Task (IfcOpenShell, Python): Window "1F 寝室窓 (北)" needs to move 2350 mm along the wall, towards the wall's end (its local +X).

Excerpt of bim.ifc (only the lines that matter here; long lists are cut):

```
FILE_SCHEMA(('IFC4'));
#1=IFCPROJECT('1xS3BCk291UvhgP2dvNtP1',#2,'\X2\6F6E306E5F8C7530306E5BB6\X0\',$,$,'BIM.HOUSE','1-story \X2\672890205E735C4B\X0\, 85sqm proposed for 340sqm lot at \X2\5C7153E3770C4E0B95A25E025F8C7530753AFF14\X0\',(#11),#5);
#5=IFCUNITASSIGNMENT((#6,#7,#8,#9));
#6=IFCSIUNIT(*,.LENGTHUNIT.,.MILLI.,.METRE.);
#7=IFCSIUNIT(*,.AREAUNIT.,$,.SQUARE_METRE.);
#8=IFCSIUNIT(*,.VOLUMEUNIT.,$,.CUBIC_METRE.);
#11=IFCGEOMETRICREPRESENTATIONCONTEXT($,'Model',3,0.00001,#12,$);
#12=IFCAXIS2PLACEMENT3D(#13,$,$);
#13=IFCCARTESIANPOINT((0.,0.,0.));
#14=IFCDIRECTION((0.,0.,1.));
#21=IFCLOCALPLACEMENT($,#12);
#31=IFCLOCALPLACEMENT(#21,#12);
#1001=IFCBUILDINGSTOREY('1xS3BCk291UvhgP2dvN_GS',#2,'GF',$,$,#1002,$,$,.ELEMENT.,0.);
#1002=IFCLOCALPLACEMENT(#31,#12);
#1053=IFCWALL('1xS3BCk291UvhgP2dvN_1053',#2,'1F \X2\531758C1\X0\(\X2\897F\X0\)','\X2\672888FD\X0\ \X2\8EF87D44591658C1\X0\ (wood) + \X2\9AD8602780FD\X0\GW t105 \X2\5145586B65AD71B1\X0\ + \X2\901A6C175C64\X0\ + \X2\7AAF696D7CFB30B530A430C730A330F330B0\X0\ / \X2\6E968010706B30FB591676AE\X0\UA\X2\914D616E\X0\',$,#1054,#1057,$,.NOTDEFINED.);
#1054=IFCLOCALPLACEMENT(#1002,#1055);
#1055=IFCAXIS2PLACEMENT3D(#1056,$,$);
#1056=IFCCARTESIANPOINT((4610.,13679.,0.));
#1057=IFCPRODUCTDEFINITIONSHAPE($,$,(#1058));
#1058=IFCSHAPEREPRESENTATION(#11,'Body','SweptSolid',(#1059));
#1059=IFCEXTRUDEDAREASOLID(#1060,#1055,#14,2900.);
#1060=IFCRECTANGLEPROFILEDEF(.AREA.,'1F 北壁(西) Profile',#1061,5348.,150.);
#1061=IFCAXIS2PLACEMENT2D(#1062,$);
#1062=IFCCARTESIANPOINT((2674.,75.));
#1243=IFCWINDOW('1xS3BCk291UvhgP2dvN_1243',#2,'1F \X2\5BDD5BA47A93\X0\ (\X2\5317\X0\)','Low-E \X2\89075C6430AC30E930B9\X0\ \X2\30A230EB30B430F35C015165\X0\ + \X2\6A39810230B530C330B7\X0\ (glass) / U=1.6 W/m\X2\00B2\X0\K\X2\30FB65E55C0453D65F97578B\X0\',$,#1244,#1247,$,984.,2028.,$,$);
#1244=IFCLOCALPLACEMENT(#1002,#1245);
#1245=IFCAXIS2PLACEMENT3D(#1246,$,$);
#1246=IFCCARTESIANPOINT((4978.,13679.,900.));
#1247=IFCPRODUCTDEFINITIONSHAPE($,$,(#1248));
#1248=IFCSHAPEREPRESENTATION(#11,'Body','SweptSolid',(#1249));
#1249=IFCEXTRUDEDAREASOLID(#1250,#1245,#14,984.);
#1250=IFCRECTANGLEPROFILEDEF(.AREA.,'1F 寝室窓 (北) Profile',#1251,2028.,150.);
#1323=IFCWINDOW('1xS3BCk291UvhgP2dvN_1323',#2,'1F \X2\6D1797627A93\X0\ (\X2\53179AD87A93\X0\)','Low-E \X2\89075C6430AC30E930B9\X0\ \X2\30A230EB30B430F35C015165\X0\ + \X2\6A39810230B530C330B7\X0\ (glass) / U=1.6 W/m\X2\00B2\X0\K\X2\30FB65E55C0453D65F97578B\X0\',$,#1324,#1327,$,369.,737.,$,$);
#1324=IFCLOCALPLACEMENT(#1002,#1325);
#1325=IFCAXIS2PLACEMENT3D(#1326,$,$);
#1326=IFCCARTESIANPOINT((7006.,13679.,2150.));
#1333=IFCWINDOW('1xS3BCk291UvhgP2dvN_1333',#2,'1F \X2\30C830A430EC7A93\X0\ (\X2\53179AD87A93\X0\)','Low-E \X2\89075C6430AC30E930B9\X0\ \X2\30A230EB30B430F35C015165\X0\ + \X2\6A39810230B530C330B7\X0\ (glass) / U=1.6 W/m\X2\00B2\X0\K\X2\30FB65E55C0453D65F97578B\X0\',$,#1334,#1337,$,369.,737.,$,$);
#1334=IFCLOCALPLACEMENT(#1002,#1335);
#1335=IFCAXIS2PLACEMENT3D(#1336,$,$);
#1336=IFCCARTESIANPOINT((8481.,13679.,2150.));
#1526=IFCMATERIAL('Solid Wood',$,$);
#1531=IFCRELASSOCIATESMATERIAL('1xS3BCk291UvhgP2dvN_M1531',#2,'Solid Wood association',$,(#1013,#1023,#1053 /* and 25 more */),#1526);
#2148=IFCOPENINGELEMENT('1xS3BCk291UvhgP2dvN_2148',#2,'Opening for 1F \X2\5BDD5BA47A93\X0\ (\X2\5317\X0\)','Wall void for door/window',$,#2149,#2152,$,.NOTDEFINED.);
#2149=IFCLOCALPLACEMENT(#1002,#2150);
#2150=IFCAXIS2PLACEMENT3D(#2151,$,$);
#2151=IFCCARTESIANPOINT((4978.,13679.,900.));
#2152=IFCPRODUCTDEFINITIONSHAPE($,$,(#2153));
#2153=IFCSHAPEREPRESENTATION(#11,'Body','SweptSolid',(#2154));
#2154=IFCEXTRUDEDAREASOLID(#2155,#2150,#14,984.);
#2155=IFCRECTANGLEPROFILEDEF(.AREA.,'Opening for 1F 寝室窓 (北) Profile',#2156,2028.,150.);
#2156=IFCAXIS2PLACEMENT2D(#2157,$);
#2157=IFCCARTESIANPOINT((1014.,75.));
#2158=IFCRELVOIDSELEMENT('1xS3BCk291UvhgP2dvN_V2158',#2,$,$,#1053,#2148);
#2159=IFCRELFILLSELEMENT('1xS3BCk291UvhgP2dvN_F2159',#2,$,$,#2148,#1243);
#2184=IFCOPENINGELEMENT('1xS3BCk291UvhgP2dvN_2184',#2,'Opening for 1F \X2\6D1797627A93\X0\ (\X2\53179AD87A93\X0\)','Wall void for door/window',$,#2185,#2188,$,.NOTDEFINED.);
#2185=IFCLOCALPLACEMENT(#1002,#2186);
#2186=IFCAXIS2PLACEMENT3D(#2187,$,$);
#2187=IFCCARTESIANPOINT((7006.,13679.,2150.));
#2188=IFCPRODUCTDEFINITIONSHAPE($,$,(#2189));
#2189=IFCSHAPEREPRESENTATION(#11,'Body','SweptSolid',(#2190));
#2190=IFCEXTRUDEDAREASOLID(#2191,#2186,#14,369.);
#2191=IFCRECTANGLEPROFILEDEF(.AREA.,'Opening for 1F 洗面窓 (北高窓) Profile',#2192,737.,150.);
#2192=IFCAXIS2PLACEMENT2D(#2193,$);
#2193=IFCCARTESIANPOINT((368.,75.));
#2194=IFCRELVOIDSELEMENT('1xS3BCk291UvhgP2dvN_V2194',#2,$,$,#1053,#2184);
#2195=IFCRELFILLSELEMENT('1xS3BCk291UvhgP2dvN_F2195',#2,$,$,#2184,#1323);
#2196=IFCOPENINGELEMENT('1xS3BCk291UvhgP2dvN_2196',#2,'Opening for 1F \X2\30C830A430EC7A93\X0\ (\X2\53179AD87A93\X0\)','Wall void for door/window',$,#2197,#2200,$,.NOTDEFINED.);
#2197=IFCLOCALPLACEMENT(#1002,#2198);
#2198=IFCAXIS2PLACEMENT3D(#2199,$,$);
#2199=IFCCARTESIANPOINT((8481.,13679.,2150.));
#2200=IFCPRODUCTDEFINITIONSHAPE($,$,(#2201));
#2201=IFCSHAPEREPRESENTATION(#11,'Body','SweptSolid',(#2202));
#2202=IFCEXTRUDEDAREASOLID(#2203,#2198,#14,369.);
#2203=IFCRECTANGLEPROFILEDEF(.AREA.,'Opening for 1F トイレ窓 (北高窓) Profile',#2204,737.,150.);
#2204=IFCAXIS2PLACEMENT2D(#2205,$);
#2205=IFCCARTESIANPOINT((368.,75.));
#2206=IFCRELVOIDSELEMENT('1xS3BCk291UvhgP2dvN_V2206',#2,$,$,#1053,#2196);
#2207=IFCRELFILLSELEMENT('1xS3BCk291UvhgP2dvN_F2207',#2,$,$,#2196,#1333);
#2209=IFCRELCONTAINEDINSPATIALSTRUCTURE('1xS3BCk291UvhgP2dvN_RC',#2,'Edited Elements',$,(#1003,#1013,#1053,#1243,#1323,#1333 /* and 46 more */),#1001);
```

```python
import ifcopenshell
import ifcopenshell.api.geometry
import ifcopenshell.util.placement
import ifcopenshell.util.unit

model = ifcopenshell.open("bim.ifc")
unit_scale = ifcopenshell.util.unit.calculate_unit_scale(model)

window = model.by_id(1243)
opening = window.FillsVoids[0].RelatingOpeningElement
wall = opening.VoidsElements[0].RelatingBuildingElement

wall_matrix = ifcopenshell.util.placement.get_local_placement(wall.ObjectPlacement)
shift = wall_matrix[:3, 0] * 2.35 / unit_scale
before = ifcopenshell.util.placement.get_local_placement(window.ObjectPlacement)[:3, 3].copy()

# The window is not placed relative to its opening, so move both.
for product in (opening, window):
    matrix = ifcopenshell.util.placement.get_local_placement(product.ObjectPlacement)
    matrix[:3, 3] += shift
    ifcopenshell.api.geometry.edit_object_placement(model, product=product, matrix=matrix, is_si=False)

after = ifcopenshell.util.placement.get_local_placement(window.ObjectPlacement)[:3, 3]
print("window moved by", (after - before).round(3) + 0.0)

model.write("bim_updated.ifc")
```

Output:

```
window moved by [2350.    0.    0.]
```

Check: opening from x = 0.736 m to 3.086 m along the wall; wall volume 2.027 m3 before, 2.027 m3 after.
